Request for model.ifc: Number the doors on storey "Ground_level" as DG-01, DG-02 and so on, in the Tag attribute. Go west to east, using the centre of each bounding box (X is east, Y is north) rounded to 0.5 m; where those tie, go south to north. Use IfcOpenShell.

First a look at what the model holds.

```python
import ifcopenshell
import ifcopenshell.util.element
import ifcopenshell.util.placement

model = ifcopenshell.open("model.ifc")
print(model.schema)
storey = next(s for s in model.by_type("IfcBuildingStorey") if s.Name == "Ground_level")
doors = [e for e in ifcopenshell.util.element.get_decomposition(storey) if e.is_a("IfcDoor")]
for e in sorted(doors, key=lambda e: e.id()):
    origin = ifcopenshell.util.placement.get_local_placement(e.ObjectPlacement)[:3, 3]
    print(e.id(), e.Tag, e.Name, origin.round(2) + 0.0, sep=" | ")
```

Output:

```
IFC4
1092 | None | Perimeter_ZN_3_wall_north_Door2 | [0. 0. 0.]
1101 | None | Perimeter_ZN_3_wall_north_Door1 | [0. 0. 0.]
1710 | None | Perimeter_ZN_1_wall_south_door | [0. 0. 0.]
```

```python
import ifcopenshell
import ifcopenshell.geom
import ifcopenshell.util.element
import ifcopenshell.util.shape

model = ifcopenshell.open("model.ifc")
settings = ifcopenshell.geom.settings()
settings.set("use-world-coords", True)


def centre(element):
    shape = ifcopenshell.geom.create_shape(settings, element)
    return ifcopenshell.util.shape.get_bbox_centroid(shape.geometry)


storey = next(s for s in model.by_type("IfcBuildingStorey") if s.Name == "Ground_level")
doors = [e for e in ifcopenshell.util.element.get_decomposition(storey) if e.is_a("IfcDoor")]

# Insertion points can sit at a corner or the storey origin, so sort by the geometry (in metres).
centres = {e: centre(e) for e in doors}
doors.sort(key=lambda e: (round(centres[e][0] / 0.5), centres[e][1]))

for i, e in enumerate(doors, start=1):
    number = f"DG-{i:02d}"
    e.Tag = number
    print(e.id(), number)

model.write("model-out.ifc")
```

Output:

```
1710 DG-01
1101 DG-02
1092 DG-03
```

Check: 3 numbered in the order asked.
